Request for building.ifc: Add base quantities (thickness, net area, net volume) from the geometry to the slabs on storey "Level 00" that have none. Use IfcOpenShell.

First a look at what the model holds.

```python
import ifcopenshell
import ifcopenshell.util.element
import ifcopenshell.util.unit

model = ifcopenshell.open("building.ifc")
print(model.schema)
for unit_type in ("LENGTHUNIT", "AREAUNIT", "VOLUMEUNIT"):
    print(unit_type, ifcopenshell.util.unit.calculate_unit_scale(model, unit_type))
storey = next(s for s in model.by_type("IfcBuildingStorey") if s.Name == "Level 00")
slabs = [e for e in ifcopenshell.util.element.get_decomposition(storey) if e.is_a("IfcSlab")]
for e in sorted(slabs, key=lambda e: e.id()):
    print(e.id(), e.is_a(), e.Name, list(ifcopenshell.util.element.get_psets(e, qtos_only=True)), sep=" | ")
```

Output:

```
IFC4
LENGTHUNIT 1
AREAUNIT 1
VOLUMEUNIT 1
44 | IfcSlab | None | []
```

```python
import ifcopenshell
import ifcopenshell.api.pset
import ifcopenshell.geom
import ifcopenshell.util.element
import ifcopenshell.util.shape
import ifcopenshell.util.unit

model = ifcopenshell.open("building.ifc")
unit_scale = ifcopenshell.util.unit.calculate_unit_scale(model)
area_scale = ifcopenshell.util.unit.calculate_unit_scale(model, "AREAUNIT")
volume_scale = ifcopenshell.util.unit.calculate_unit_scale(model, "VOLUMEUNIT")
settings = ifcopenshell.geom.settings()

storey = next(s for s in model.by_type("IfcBuildingStorey") if s.Name == "Level 00")
slabs = [e for e in ifcopenshell.util.element.get_decomposition(storey) if e.is_a("IfcSlab")]

for e in sorted(slabs, key=lambda e: e.id()):
    if ifcopenshell.util.element.get_psets(e, qtos_only=True, should_inherit=False):
        continue
    # Geometry comes back in metres, in the element's own axes.
    shape = ifcopenshell.geom.create_shape(settings, e)
    values = {
        "Width": ifcopenshell.util.shape.get_z(shape.geometry) / unit_scale,
        "NetArea": ifcopenshell.util.shape.get_footprint_area(shape.geometry) / area_scale,
        "NetVolume": ifcopenshell.util.shape.get_volume(shape.geometry) / volume_scale,
    }
    qto = ifcopenshell.api.pset.add_qto(model, product=e, name="Qto_SlabBaseQuantities")
    ifcopenshell.api.pset.edit_qto(model, qto=qto, properties=values)
    print(e.id(), {k: round(v, 3) for k, v in values.items()})

model.write("building-out.ifc")
```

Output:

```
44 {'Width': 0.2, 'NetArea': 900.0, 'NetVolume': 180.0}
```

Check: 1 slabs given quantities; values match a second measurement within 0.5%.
